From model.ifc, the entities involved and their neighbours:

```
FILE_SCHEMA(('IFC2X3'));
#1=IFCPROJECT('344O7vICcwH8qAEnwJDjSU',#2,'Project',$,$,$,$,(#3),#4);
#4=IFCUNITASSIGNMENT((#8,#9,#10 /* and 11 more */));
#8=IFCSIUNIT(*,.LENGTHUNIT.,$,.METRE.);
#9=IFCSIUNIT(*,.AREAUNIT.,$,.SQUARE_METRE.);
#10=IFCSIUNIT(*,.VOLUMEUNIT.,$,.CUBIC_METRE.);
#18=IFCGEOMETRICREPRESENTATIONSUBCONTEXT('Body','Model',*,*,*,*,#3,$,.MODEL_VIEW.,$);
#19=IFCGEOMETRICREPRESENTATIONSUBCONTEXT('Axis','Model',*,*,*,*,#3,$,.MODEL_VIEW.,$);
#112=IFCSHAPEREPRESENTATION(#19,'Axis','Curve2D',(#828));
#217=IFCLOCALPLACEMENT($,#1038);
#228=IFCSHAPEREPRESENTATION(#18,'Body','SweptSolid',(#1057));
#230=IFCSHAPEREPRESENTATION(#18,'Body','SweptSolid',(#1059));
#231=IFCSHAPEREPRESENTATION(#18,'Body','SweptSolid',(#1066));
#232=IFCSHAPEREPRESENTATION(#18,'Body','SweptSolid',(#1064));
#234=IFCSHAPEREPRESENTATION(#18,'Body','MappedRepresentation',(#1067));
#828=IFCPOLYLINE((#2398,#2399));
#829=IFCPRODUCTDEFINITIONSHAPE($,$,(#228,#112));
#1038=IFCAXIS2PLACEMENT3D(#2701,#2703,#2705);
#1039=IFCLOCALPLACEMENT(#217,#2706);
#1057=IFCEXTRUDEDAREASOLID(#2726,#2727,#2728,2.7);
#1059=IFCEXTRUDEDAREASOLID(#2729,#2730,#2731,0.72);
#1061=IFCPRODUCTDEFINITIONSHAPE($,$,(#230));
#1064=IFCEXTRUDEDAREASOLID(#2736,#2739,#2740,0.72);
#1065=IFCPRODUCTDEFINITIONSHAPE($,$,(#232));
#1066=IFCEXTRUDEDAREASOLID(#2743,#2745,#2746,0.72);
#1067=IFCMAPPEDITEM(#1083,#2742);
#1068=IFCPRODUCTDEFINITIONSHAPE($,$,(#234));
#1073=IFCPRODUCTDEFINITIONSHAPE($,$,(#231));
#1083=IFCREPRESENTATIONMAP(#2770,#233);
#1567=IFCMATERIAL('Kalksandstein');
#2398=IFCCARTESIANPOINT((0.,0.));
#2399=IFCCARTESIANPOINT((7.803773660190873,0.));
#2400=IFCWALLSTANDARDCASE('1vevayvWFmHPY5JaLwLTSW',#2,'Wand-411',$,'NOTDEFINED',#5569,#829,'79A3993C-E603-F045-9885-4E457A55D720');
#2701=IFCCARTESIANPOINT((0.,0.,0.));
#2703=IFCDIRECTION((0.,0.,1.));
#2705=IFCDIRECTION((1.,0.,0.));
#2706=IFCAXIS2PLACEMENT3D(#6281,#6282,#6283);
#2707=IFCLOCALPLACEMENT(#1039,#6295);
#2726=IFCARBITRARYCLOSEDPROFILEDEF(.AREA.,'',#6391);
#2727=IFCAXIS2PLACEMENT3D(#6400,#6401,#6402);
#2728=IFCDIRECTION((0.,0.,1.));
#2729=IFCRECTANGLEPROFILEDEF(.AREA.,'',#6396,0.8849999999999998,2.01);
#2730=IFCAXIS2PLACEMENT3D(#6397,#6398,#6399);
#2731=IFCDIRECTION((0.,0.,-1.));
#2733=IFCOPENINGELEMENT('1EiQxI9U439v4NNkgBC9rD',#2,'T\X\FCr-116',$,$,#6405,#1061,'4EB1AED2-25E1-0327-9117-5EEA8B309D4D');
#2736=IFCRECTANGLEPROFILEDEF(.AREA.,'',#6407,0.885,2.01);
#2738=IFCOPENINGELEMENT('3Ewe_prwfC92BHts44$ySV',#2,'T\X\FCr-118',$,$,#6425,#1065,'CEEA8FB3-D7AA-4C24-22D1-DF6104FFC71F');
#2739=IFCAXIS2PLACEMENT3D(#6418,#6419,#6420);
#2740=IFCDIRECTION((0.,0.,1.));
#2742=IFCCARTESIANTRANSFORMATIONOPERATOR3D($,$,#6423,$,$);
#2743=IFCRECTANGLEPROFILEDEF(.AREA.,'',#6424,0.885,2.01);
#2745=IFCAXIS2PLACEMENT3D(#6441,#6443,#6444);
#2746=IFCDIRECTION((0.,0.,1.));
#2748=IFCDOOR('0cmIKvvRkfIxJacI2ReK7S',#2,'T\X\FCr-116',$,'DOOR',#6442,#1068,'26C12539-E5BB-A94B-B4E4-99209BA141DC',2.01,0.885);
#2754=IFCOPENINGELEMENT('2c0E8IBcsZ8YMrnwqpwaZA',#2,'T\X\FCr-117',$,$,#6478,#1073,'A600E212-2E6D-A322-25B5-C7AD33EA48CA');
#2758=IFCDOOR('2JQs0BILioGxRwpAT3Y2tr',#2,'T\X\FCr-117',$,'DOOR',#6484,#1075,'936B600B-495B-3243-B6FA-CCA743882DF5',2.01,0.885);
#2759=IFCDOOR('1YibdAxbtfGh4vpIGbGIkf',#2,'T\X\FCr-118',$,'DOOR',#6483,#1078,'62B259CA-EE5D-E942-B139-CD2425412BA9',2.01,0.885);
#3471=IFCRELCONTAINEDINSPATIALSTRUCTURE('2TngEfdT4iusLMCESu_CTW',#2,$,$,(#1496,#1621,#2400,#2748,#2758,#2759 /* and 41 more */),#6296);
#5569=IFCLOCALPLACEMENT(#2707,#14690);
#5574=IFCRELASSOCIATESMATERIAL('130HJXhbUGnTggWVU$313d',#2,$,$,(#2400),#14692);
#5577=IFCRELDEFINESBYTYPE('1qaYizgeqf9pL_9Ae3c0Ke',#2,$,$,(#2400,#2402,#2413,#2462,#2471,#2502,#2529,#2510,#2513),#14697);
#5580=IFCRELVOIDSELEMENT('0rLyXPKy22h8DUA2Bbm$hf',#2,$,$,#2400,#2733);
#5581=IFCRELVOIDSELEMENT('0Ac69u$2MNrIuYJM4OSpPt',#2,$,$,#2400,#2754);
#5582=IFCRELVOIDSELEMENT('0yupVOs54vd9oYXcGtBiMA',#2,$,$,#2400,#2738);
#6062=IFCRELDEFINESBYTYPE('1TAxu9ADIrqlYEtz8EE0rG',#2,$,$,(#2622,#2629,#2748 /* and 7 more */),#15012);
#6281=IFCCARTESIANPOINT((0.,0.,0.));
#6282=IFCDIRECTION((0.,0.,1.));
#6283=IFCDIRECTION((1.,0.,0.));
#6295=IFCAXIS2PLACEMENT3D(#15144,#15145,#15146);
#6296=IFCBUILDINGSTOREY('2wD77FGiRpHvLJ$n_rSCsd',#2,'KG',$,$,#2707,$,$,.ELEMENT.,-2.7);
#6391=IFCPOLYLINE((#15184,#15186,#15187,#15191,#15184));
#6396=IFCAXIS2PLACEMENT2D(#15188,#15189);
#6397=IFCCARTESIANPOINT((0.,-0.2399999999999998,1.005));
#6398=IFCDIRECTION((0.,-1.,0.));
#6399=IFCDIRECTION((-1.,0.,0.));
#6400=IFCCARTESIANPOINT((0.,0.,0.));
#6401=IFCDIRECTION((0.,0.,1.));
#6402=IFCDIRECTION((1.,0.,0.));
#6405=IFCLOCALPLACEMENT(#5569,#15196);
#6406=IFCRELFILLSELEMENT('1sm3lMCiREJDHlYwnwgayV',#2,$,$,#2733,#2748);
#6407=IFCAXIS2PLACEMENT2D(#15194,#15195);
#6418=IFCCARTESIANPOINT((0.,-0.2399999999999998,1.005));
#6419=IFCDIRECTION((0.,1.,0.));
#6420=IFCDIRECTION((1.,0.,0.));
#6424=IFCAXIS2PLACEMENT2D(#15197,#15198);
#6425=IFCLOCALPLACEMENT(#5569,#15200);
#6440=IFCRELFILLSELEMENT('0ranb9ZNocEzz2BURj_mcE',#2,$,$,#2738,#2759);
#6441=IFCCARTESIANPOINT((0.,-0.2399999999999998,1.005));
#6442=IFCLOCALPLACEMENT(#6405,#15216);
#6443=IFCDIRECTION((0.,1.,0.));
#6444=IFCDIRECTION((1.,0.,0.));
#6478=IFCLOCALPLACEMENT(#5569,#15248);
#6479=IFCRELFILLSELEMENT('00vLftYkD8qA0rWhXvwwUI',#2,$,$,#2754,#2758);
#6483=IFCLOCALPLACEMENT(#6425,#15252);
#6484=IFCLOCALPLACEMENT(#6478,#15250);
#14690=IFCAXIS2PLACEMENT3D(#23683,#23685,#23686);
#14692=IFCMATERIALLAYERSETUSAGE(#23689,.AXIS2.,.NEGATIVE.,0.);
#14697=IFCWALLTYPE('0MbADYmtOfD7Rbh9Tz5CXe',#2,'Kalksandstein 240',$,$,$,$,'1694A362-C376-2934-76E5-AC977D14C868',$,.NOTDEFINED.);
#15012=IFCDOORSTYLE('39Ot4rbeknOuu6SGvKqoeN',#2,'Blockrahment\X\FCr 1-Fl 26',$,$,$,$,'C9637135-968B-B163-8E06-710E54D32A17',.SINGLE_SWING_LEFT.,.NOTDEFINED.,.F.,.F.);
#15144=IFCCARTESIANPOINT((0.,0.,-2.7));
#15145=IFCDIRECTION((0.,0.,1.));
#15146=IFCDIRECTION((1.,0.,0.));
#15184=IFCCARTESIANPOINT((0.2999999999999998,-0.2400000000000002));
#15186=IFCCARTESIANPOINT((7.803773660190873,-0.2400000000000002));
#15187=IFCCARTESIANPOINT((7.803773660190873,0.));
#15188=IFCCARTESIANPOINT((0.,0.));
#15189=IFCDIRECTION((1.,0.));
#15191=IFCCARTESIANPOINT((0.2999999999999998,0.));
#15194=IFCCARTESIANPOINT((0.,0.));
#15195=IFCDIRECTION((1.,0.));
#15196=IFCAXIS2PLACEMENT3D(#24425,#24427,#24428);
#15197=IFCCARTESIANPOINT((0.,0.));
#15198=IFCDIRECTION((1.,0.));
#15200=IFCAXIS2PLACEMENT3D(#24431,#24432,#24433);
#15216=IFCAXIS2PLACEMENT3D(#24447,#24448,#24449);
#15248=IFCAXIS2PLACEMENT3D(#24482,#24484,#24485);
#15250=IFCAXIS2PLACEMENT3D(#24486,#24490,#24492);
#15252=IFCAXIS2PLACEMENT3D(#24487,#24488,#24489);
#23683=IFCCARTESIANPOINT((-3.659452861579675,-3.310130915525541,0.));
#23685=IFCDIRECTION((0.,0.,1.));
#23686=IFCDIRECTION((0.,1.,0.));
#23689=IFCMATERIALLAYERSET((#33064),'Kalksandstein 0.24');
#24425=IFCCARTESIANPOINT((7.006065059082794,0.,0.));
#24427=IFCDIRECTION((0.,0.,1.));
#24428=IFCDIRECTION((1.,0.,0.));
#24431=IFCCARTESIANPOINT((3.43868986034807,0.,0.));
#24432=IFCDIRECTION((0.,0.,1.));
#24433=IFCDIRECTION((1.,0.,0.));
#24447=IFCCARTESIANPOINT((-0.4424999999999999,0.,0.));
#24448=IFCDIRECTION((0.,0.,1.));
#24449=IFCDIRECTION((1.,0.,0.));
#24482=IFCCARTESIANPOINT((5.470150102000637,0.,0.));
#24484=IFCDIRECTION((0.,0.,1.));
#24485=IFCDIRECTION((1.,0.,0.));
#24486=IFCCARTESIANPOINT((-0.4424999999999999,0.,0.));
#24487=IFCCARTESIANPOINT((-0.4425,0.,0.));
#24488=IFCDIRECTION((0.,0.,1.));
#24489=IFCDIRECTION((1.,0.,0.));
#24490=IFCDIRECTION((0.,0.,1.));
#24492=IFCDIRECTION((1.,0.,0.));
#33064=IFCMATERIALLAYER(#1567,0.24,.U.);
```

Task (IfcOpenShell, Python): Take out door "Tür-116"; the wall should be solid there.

```python
import ifcopenshell
import ifcopenshell.api.feature
import ifcopenshell.api.root
import ifcopenshell.geom
import ifcopenshell.util.shape

model = ifcopenshell.open("model.ifc")
settings = ifcopenshell.geom.settings()


def volume(element):
    """Net volume in cubic metres, openings subtracted."""
    shape = ifcopenshell.geom.create_shape(settings, element)
    return ifcopenshell.util.shape.get_volume(shape.geometry)


door = model.by_id(2748)
opening = door.FillsVoids[0].RelatingOpeningElement
wall = opening.VoidsElements[0].RelatingBuildingElement
before = volume(wall)

ifcopenshell.api.root.remove_product(model, product=door)
ifcopenshell.api.feature.remove_feature(model, feature=opening)

after = volume(wall)

print(f"wall volume {before:.3f} -> {after:.3f} m3")

model.write("model-out.ifc")
```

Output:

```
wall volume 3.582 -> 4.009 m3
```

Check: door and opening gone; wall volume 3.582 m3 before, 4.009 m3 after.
